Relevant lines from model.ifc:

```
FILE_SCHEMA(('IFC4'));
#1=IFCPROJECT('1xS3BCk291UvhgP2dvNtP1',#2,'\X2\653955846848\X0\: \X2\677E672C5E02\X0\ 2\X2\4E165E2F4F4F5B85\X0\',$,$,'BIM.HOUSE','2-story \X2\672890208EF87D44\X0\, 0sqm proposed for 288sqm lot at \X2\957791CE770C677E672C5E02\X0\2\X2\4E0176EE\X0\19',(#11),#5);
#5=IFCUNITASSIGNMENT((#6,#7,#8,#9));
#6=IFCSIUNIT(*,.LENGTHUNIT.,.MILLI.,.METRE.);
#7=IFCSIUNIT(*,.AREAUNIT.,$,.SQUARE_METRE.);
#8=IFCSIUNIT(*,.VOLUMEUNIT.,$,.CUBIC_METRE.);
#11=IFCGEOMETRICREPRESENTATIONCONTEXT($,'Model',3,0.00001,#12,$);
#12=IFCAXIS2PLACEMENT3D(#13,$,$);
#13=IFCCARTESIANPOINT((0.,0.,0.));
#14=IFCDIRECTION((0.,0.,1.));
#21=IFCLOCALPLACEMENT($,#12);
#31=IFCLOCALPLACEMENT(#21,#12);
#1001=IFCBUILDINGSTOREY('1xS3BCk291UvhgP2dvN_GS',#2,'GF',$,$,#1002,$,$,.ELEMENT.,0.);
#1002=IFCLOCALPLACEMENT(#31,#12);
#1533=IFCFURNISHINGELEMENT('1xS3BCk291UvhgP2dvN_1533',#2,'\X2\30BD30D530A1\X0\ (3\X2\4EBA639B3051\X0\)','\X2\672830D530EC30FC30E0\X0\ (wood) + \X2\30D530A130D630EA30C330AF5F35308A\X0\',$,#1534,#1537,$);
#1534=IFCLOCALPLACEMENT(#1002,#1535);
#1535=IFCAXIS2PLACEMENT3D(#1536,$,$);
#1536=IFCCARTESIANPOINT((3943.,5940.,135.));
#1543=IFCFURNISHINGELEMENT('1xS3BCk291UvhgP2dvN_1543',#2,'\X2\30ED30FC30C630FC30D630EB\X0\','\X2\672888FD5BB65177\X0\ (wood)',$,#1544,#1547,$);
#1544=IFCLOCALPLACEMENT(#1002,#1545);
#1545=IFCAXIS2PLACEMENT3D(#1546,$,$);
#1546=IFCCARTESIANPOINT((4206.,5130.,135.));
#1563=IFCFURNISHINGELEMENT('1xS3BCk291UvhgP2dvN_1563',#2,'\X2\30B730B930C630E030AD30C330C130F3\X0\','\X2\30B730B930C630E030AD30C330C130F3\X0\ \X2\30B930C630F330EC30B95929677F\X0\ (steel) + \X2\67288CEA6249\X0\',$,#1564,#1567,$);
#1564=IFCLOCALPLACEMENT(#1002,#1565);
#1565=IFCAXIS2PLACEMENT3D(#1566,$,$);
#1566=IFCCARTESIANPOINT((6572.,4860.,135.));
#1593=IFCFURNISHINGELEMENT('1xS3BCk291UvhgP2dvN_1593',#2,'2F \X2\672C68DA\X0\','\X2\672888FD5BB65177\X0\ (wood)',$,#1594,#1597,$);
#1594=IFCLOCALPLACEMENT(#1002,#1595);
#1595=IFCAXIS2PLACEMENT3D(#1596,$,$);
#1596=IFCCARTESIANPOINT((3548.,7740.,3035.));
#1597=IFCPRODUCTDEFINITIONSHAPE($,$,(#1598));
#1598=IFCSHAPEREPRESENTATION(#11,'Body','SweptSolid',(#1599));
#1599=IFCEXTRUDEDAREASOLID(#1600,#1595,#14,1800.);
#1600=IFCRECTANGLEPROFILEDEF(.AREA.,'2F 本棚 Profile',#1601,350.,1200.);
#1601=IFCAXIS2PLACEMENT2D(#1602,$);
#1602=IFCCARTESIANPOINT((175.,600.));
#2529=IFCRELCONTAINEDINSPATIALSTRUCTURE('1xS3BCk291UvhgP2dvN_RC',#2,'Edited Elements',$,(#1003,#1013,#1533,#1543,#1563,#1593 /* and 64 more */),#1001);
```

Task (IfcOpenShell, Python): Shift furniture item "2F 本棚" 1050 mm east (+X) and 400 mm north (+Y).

```python
import ifcopenshell
import ifcopenshell.api.geometry
import ifcopenshell.util.placement

model = ifcopenshell.open("model.ifc")

item = model.by_id(1593)
matrix = ifcopenshell.util.placement.get_local_placement(item.ObjectPlacement)
matrix[0, 3] += 1050.0
matrix[1, 3] += 400.0
ifcopenshell.api.geometry.edit_object_placement(model, product=item, matrix=matrix, is_si=False)

print(ifcopenshell.util.placement.get_local_placement(item.ObjectPlacement).round(3) + 0.0)

model.write("model_updated.ifc")
```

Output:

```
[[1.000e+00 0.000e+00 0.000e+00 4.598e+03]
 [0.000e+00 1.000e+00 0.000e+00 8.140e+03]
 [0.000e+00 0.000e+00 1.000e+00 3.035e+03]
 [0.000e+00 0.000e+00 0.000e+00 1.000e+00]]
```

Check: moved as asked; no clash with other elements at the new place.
